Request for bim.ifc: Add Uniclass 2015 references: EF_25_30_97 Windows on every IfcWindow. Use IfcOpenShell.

First a look at what the model holds.

```python
import ifcopenshell

model = ifcopenshell.open("bim.ifc")
print(model.schema)
print("classifications:", [c.Name for c in model.by_type("IfcClassification")])
for ifc_class in ("IfcDoor", "IfcRoof", "IfcStair", "IfcWall", "IfcWindow"):
    print(ifc_class, len(model.by_type(ifc_class)))
```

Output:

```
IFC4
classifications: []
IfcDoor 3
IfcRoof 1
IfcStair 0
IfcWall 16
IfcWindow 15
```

```python
import ifcopenshell
import ifcopenshell.api.classification

model = ifcopenshell.open("bim.ifc")

system = ifcopenshell.api.classification.add_classification(model, classification="Uniclass 2015")

codes = {
    "IfcWindow": ("EF_25_30_97", "Windows"),
}
for ifc_class, (code, name) in codes.items():
    products = model.by_type(ifc_class)
    ifcopenshell.api.classification.add_reference(
        model, products=products, classification=system, identification=code, name=name
    )
    print(code, len(products))

model.write("bim_rev.ifc")
```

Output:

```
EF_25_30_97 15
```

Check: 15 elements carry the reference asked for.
